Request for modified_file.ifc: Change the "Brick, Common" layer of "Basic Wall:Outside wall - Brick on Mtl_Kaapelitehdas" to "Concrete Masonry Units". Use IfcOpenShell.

First a look at what the model holds.

```python
import ifcopenshell
import ifcopenshell.util.element

model = ifcopenshell.open("modified_file.ifc")
print(model.schema)
for layer_set in model.by_type("IfcMaterialLayerSet"):
    if layer_set.LayerSetName == "Basic Wall:Outside wall - Brick on Mtl_Kaapelitehdas":
        for layer in layer_set.MaterialLayers:
            print(layer.id(), layer.Material and layer.Material.Name, layer.LayerThickness, sep=" | ")
        print(len(ifcopenshell.util.element.get_elements_by_material(model, layer_set)), "elements and types use it")
print(sorted(m.Name for m in model.by_type("IfcMaterial") if m.Name)[:60])
```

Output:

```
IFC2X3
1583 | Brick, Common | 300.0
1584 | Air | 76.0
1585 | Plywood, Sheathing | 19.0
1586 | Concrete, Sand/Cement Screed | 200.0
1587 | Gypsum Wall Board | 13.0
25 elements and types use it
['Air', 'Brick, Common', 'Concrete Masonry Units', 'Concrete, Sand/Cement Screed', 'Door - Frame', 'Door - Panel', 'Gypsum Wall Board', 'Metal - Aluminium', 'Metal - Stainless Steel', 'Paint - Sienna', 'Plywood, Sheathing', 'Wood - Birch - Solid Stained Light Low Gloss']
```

```python
import ifcopenshell
import ifcopenshell.api.material

model = ifcopenshell.open("modified_file.ifc")

layer_set = next(s for s in model.by_type("IfcMaterialLayerSet") if s.LayerSetName == "Basic Wall:Outside wall - Brick on Mtl_Kaapelitehdas")
layer = next(l for l in layer_set.MaterialLayers if l.Material and l.Material.Name == "Brick, Common")
material = next(m for m in model.by_type("IfcMaterial") if m.Name == "Concrete Masonry Units")

# Point this one layer at the other material; renaming the old one would change it everywhere.
ifcopenshell.api.material.edit_layer(model, layer=layer, attributes={}, material=material)

print([l.Material.Name if l.Material else None for l in layer_set.MaterialLayers])

model.write("modified_file-out.ifc")
```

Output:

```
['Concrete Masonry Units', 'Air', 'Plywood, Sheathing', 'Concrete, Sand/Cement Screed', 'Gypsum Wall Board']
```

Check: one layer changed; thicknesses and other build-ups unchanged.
